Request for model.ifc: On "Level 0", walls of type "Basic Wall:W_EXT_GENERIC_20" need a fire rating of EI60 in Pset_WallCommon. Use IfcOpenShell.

First a look at what the model holds.

```python
import ifcopenshell
import ifcopenshell.util.element

model = ifcopenshell.open("model.ifc")
print(model.schema)
storey = next(s for s in model.by_type("IfcBuildingStorey") if s.Name == "Level 0")
walls = [e for e in ifcopenshell.util.element.get_decomposition(storey) if e.is_a("IfcWall")]
seen = {}
for e in walls:
    element_type = ifcopenshell.util.element.get_type(e)
    key = (element_type.Name if element_type != e and element_type else None, ifcopenshell.util.element.get_pset(e, "Pset_WallCommon", "FireRating"))
    seen[key] = seen.get(key, 0) + 1
for (name, value), count in sorted(seen.items(), key=str):
    print(count, "x", name, "|", value)
```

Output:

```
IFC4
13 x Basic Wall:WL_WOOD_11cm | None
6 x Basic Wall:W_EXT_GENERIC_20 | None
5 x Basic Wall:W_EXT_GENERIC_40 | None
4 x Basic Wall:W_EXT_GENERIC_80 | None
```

```python
import ifcopenshell
import ifcopenshell.api.pset
import ifcopenshell.util.element

model = ifcopenshell.open("model.ifc")

storey = next(s for s in model.by_type("IfcBuildingStorey") if s.Name == "Level 0")
walls = [e for e in ifcopenshell.util.element.get_decomposition(storey) if e.is_a("IfcWall")]

count = 0
for e in walls:
    element_type = ifcopenshell.util.element.get_type(e)
    if element_type in (None, e) or element_type.Name != "Basic Wall:W_EXT_GENERIC_20":
        continue
    # add_pset returns the element's existing set when there is one.
    pset = ifcopenshell.api.pset.add_pset(model, product=e, name="Pset_WallCommon")
    ifcopenshell.api.pset.edit_pset(model, pset=pset, properties={"FireRating": "EI60"})
    count += 1

print(count, "walls updated")

model.write("model_rev.ifc")
```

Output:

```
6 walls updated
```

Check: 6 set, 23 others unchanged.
